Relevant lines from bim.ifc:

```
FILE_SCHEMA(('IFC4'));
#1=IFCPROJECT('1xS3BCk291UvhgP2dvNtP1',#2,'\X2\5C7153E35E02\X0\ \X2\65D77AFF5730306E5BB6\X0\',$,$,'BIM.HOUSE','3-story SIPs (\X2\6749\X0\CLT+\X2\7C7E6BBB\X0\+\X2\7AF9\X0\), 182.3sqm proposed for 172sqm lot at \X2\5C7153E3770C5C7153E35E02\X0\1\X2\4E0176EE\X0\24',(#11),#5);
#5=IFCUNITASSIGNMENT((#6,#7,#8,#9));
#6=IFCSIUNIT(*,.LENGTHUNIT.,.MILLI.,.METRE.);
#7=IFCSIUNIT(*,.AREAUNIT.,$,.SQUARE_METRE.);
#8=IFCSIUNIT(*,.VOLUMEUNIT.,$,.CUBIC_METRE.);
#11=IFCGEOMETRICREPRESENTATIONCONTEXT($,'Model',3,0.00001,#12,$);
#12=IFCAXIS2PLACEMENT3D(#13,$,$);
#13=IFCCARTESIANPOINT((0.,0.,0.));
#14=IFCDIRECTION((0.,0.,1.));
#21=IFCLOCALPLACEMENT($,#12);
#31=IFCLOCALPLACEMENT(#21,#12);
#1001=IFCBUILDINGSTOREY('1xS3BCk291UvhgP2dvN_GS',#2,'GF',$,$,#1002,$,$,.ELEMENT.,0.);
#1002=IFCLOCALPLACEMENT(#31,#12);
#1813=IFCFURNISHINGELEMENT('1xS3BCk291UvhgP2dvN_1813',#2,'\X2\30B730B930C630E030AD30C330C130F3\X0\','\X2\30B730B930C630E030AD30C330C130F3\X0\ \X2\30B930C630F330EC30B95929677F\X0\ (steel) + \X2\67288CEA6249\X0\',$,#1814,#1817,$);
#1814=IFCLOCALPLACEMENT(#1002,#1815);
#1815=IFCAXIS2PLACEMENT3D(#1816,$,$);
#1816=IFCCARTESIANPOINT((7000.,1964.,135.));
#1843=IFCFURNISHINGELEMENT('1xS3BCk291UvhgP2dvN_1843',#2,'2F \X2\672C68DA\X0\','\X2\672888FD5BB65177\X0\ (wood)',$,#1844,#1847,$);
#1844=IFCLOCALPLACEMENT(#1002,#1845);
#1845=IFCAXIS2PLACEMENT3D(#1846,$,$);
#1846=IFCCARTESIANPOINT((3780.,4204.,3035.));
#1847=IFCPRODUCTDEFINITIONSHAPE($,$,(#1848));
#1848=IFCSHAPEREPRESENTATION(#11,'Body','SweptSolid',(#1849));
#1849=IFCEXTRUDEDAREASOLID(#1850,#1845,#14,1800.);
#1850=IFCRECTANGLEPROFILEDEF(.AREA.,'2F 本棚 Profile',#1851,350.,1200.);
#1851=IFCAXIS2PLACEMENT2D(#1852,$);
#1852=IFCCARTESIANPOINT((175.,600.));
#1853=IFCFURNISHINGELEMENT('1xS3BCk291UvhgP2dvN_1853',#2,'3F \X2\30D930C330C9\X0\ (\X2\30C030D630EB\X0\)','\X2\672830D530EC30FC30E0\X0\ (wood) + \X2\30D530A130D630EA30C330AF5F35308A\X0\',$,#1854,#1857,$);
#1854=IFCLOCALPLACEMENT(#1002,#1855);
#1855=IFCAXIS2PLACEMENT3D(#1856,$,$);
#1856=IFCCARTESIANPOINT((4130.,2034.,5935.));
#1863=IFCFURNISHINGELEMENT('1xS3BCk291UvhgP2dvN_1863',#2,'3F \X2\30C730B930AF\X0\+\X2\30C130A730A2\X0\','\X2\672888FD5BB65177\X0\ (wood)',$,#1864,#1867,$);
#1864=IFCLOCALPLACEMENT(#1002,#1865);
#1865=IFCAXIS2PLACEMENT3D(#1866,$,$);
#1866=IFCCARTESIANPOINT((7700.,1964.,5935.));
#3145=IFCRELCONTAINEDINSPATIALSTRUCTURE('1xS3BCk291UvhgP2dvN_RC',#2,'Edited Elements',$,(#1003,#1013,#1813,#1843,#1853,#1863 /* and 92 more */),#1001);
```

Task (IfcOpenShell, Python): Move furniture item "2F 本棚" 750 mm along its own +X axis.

```python
import ifcopenshell
import ifcopenshell.api.geometry
import ifcopenshell.util.placement
import ifcopenshell.util.unit

model = ifcopenshell.open("bim.ifc")
unit_scale = ifcopenshell.util.unit.calculate_unit_scale(model)

item = model.by_id(1843)
matrix = ifcopenshell.util.placement.get_local_placement(item.ObjectPlacement)
matrix[:3, 3] += matrix[:3, 0] * 0.75 / unit_scale
ifcopenshell.api.geometry.edit_object_placement(model, product=item, matrix=matrix, is_si=False)

print(ifcopenshell.util.placement.get_local_placement(item.ObjectPlacement).round(3) + 0.0)

model.write("bim_v2.ifc")
```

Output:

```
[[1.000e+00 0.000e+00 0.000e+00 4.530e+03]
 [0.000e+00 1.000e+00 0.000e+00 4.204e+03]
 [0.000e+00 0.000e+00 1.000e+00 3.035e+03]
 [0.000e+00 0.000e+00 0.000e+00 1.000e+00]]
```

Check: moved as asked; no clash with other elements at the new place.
